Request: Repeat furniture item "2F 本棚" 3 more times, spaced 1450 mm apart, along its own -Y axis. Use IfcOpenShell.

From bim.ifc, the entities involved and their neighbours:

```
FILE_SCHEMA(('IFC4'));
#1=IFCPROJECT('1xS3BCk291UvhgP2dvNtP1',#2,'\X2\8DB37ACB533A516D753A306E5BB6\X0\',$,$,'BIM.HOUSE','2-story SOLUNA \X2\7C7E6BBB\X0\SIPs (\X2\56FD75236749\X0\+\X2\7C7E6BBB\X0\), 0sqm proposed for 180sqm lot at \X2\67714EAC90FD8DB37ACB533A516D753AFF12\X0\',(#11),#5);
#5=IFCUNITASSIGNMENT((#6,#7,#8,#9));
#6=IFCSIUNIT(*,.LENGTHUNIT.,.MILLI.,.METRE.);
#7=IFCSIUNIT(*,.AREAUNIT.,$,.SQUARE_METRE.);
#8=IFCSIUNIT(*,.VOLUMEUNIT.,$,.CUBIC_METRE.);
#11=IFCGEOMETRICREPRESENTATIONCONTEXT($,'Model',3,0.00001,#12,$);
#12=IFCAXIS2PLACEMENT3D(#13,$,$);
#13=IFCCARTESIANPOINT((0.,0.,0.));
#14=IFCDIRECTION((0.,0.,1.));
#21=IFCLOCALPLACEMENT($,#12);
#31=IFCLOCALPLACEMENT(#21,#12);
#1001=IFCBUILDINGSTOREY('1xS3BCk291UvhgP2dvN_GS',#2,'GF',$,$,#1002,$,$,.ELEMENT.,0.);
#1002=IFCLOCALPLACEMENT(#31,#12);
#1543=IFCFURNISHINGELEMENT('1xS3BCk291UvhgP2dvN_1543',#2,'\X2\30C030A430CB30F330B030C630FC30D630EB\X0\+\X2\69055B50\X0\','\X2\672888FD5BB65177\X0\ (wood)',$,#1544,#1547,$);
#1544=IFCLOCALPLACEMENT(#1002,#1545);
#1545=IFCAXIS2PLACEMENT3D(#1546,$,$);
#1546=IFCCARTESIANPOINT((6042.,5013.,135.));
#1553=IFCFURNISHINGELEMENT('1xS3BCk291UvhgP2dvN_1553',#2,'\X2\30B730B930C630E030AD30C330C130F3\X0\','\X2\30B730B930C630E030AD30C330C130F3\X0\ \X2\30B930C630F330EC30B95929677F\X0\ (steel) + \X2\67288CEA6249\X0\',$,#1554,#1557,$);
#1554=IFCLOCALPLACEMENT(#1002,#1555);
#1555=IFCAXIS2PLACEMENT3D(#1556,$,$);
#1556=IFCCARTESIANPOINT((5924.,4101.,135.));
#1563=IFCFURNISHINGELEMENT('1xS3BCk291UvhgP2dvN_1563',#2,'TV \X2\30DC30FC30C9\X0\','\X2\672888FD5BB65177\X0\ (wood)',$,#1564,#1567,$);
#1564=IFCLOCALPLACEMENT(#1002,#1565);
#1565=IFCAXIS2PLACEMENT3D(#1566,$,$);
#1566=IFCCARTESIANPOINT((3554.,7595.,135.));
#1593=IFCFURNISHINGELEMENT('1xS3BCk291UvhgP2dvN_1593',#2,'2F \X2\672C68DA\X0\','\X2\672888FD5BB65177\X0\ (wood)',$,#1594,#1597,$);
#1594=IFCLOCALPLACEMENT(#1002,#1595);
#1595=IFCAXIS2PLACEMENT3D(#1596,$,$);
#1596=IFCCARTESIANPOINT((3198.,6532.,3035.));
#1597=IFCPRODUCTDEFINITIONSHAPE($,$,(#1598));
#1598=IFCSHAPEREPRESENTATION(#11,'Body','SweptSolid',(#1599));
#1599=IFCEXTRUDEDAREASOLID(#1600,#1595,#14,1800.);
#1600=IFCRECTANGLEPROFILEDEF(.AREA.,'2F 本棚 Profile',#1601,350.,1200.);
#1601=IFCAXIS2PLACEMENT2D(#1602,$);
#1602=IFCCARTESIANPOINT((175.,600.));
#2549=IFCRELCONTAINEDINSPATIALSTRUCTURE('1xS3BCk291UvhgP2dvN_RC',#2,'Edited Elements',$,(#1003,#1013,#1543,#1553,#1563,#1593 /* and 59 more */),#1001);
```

```python
import ifcopenshell
import ifcopenshell.api.geometry
import ifcopenshell.api.root
import ifcopenshell.util.element
import ifcopenshell.util.placement
import ifcopenshell.util.unit

model = ifcopenshell.open("bim.ifc")
unit_scale = ifcopenshell.util.unit.calculate_unit_scale(model)


def reuse_history(source, copy):
    """copy_class also copies each property set's owner history, people and application; keep the originals."""
    for rel in copy.IsDefinedBy:
        if rel.is_a("IfcRelDefinesByProperties") and (history := rel.RelatingPropertyDefinition.OwnerHistory):
            rel.RelatingPropertyDefinition.OwnerHistory = source.OwnerHistory
            ifcopenshell.util.element.remove_deep2(model, history)


source = model.by_guid("1xS3BCk291UvhgP2dvN_1593")
base = ifcopenshell.util.placement.get_local_placement(source.ObjectPlacement)
step = -base[:3, 1] * 1.45 / unit_scale

for i in range(1, 4):
    copy = ifcopenshell.api.root.copy_class(model, product=source)
    copy.Representation = ifcopenshell.util.element.copy_deep(
        model, source.Representation, exclude=["IfcGeometricRepresentationContext", "IfcRepresentationMap"]
    )
    reuse_history(source, copy)
    matrix = base.copy()
    matrix[:3, 3] += i * step
    print("added at", matrix[:3, 3].round(3) + 0.0)
    ifcopenshell.api.geometry.edit_object_placement(model, product=copy, matrix=matrix, is_si=False)

model.write("bim_edited.ifc")
```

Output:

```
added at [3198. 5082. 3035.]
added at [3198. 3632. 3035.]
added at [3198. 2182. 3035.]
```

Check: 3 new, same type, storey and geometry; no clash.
